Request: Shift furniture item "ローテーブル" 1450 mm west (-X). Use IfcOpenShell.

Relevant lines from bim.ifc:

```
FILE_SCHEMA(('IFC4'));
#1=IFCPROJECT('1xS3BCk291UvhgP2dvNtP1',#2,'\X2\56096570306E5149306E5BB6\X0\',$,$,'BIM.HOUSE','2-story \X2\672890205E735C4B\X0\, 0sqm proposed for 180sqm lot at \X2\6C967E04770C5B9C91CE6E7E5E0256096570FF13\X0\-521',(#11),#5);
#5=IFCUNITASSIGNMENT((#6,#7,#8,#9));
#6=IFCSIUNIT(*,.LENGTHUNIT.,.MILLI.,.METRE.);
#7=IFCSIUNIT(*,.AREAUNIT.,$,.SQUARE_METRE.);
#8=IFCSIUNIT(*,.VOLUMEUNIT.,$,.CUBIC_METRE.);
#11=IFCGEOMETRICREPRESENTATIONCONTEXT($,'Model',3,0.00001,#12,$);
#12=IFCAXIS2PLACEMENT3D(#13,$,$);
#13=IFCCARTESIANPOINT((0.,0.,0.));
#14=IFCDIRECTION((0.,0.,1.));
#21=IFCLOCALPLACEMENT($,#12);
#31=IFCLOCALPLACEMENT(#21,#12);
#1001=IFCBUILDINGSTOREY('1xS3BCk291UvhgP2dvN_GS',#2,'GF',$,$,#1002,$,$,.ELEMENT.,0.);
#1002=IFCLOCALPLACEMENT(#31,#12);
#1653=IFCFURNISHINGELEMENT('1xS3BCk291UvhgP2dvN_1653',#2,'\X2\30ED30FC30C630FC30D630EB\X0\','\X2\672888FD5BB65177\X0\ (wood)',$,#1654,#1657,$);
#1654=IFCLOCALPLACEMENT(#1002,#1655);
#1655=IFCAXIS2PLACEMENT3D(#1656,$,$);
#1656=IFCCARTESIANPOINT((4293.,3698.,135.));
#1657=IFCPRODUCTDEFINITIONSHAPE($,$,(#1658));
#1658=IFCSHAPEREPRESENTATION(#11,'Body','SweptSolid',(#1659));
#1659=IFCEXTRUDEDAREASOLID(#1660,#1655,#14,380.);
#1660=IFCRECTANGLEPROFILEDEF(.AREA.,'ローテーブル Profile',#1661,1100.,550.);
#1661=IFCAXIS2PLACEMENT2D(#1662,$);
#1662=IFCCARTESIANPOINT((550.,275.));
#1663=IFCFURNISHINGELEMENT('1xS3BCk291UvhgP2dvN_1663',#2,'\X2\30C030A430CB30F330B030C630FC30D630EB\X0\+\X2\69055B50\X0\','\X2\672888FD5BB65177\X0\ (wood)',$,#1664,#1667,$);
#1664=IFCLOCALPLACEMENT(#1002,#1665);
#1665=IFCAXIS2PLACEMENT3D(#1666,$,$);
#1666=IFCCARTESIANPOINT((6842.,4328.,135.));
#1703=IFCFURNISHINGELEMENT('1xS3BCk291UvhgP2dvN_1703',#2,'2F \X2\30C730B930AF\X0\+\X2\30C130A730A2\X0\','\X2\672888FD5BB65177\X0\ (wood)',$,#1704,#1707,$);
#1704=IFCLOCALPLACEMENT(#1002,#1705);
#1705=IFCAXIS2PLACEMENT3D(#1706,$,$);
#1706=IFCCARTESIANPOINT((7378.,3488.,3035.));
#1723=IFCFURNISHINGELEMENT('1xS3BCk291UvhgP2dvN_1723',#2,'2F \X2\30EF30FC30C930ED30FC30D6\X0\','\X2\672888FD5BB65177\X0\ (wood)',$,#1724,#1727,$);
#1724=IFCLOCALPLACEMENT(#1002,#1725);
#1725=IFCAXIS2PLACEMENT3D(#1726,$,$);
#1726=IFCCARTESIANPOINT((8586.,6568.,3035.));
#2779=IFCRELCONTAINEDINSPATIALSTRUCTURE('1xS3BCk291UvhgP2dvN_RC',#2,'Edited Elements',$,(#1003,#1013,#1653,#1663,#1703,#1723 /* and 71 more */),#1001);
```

```python
import ifcopenshell
import ifcopenshell.api.geometry
import ifcopenshell.util.placement
import ifcopenshell.util.unit

model = ifcopenshell.open("bim.ifc")
unit_scale = ifcopenshell.util.unit.calculate_unit_scale(model)

item = model.by_guid("1xS3BCk291UvhgP2dvN_1653")
matrix = ifcopenshell.util.placement.get_local_placement(item.ObjectPlacement)
matrix[0, 3] -= 1.45 / unit_scale
ifcopenshell.api.geometry.edit_object_placement(model, product=item, matrix=matrix, is_si=False)

print(ifcopenshell.util.placement.get_local_placement(item.ObjectPlacement).round(3) + 0.0)

model.write("bim_rev.ifc")
```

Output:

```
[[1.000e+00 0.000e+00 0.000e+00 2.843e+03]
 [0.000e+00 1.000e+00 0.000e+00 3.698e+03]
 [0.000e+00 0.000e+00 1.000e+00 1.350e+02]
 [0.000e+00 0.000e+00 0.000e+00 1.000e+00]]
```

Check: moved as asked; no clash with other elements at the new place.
